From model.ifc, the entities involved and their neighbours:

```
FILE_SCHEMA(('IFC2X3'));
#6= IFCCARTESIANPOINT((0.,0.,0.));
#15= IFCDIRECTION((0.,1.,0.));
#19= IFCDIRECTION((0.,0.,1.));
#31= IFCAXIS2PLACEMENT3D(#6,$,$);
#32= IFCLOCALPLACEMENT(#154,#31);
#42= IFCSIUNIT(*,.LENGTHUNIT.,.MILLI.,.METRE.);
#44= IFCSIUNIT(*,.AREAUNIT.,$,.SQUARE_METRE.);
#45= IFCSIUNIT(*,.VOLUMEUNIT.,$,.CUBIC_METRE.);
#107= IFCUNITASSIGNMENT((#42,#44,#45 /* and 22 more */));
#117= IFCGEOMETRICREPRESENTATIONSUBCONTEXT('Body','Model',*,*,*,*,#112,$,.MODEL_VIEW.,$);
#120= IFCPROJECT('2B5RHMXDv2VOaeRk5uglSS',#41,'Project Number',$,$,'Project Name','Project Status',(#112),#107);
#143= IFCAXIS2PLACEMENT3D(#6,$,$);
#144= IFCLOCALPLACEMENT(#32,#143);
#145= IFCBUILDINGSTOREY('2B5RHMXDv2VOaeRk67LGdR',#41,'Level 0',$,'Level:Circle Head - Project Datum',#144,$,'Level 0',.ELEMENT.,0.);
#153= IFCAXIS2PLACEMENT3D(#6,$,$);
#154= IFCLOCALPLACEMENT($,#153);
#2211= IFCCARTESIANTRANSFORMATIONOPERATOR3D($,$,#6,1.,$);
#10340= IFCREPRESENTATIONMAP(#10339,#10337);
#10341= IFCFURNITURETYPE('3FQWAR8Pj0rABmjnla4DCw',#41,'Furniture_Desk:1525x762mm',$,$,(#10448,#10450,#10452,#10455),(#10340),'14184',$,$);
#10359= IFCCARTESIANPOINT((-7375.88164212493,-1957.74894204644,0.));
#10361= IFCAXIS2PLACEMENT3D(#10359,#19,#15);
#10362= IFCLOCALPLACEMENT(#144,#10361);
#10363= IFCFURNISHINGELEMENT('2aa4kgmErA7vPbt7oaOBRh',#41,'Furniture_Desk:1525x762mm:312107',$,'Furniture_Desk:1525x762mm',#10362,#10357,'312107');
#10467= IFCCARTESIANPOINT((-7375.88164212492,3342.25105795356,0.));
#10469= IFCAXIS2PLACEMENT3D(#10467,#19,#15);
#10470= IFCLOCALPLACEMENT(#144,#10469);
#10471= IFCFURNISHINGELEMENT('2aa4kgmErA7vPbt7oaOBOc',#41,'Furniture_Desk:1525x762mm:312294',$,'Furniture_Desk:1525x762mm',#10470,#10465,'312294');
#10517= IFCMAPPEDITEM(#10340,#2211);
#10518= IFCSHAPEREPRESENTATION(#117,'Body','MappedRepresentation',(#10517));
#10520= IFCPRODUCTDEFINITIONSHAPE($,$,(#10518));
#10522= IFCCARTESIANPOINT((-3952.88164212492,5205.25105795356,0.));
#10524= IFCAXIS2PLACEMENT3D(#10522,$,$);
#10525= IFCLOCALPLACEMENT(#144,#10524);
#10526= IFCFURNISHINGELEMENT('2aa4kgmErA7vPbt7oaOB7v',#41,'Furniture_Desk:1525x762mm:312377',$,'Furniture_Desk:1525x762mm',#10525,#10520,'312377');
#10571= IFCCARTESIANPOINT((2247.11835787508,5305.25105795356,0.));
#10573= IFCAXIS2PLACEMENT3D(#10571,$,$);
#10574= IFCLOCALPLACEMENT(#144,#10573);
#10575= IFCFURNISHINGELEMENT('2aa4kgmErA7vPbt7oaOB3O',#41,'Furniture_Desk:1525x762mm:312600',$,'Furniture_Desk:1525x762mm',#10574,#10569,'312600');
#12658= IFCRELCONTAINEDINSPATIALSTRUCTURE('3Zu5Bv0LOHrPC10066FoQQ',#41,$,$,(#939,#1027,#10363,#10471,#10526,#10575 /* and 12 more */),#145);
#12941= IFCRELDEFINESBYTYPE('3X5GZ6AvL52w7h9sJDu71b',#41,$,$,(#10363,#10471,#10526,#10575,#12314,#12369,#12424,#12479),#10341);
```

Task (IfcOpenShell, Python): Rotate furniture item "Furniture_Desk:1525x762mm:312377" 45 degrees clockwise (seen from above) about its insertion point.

```python
import ifcopenshell
import ifcopenshell.api.geometry
import ifcopenshell.util.placement

model = ifcopenshell.open("model.ifc")

item = model.by_guid("2aa4kgmErA7vPbt7oaOB7v")
matrix = ifcopenshell.util.placement.get_local_placement(item.ObjectPlacement)
matrix = matrix @ ifcopenshell.util.placement.rotation(-45, "Z")
ifcopenshell.api.geometry.edit_object_placement(model, product=item, matrix=matrix, is_si=False)

print(ifcopenshell.util.placement.get_local_placement(item.ObjectPlacement).round(3) + 0.0)

model.write("model_v2.ifc")
```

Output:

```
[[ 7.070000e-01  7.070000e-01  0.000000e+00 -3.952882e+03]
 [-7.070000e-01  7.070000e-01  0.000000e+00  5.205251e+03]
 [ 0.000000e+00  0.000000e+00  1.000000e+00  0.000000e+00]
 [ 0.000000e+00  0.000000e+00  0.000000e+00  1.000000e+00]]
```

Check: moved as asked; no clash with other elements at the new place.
